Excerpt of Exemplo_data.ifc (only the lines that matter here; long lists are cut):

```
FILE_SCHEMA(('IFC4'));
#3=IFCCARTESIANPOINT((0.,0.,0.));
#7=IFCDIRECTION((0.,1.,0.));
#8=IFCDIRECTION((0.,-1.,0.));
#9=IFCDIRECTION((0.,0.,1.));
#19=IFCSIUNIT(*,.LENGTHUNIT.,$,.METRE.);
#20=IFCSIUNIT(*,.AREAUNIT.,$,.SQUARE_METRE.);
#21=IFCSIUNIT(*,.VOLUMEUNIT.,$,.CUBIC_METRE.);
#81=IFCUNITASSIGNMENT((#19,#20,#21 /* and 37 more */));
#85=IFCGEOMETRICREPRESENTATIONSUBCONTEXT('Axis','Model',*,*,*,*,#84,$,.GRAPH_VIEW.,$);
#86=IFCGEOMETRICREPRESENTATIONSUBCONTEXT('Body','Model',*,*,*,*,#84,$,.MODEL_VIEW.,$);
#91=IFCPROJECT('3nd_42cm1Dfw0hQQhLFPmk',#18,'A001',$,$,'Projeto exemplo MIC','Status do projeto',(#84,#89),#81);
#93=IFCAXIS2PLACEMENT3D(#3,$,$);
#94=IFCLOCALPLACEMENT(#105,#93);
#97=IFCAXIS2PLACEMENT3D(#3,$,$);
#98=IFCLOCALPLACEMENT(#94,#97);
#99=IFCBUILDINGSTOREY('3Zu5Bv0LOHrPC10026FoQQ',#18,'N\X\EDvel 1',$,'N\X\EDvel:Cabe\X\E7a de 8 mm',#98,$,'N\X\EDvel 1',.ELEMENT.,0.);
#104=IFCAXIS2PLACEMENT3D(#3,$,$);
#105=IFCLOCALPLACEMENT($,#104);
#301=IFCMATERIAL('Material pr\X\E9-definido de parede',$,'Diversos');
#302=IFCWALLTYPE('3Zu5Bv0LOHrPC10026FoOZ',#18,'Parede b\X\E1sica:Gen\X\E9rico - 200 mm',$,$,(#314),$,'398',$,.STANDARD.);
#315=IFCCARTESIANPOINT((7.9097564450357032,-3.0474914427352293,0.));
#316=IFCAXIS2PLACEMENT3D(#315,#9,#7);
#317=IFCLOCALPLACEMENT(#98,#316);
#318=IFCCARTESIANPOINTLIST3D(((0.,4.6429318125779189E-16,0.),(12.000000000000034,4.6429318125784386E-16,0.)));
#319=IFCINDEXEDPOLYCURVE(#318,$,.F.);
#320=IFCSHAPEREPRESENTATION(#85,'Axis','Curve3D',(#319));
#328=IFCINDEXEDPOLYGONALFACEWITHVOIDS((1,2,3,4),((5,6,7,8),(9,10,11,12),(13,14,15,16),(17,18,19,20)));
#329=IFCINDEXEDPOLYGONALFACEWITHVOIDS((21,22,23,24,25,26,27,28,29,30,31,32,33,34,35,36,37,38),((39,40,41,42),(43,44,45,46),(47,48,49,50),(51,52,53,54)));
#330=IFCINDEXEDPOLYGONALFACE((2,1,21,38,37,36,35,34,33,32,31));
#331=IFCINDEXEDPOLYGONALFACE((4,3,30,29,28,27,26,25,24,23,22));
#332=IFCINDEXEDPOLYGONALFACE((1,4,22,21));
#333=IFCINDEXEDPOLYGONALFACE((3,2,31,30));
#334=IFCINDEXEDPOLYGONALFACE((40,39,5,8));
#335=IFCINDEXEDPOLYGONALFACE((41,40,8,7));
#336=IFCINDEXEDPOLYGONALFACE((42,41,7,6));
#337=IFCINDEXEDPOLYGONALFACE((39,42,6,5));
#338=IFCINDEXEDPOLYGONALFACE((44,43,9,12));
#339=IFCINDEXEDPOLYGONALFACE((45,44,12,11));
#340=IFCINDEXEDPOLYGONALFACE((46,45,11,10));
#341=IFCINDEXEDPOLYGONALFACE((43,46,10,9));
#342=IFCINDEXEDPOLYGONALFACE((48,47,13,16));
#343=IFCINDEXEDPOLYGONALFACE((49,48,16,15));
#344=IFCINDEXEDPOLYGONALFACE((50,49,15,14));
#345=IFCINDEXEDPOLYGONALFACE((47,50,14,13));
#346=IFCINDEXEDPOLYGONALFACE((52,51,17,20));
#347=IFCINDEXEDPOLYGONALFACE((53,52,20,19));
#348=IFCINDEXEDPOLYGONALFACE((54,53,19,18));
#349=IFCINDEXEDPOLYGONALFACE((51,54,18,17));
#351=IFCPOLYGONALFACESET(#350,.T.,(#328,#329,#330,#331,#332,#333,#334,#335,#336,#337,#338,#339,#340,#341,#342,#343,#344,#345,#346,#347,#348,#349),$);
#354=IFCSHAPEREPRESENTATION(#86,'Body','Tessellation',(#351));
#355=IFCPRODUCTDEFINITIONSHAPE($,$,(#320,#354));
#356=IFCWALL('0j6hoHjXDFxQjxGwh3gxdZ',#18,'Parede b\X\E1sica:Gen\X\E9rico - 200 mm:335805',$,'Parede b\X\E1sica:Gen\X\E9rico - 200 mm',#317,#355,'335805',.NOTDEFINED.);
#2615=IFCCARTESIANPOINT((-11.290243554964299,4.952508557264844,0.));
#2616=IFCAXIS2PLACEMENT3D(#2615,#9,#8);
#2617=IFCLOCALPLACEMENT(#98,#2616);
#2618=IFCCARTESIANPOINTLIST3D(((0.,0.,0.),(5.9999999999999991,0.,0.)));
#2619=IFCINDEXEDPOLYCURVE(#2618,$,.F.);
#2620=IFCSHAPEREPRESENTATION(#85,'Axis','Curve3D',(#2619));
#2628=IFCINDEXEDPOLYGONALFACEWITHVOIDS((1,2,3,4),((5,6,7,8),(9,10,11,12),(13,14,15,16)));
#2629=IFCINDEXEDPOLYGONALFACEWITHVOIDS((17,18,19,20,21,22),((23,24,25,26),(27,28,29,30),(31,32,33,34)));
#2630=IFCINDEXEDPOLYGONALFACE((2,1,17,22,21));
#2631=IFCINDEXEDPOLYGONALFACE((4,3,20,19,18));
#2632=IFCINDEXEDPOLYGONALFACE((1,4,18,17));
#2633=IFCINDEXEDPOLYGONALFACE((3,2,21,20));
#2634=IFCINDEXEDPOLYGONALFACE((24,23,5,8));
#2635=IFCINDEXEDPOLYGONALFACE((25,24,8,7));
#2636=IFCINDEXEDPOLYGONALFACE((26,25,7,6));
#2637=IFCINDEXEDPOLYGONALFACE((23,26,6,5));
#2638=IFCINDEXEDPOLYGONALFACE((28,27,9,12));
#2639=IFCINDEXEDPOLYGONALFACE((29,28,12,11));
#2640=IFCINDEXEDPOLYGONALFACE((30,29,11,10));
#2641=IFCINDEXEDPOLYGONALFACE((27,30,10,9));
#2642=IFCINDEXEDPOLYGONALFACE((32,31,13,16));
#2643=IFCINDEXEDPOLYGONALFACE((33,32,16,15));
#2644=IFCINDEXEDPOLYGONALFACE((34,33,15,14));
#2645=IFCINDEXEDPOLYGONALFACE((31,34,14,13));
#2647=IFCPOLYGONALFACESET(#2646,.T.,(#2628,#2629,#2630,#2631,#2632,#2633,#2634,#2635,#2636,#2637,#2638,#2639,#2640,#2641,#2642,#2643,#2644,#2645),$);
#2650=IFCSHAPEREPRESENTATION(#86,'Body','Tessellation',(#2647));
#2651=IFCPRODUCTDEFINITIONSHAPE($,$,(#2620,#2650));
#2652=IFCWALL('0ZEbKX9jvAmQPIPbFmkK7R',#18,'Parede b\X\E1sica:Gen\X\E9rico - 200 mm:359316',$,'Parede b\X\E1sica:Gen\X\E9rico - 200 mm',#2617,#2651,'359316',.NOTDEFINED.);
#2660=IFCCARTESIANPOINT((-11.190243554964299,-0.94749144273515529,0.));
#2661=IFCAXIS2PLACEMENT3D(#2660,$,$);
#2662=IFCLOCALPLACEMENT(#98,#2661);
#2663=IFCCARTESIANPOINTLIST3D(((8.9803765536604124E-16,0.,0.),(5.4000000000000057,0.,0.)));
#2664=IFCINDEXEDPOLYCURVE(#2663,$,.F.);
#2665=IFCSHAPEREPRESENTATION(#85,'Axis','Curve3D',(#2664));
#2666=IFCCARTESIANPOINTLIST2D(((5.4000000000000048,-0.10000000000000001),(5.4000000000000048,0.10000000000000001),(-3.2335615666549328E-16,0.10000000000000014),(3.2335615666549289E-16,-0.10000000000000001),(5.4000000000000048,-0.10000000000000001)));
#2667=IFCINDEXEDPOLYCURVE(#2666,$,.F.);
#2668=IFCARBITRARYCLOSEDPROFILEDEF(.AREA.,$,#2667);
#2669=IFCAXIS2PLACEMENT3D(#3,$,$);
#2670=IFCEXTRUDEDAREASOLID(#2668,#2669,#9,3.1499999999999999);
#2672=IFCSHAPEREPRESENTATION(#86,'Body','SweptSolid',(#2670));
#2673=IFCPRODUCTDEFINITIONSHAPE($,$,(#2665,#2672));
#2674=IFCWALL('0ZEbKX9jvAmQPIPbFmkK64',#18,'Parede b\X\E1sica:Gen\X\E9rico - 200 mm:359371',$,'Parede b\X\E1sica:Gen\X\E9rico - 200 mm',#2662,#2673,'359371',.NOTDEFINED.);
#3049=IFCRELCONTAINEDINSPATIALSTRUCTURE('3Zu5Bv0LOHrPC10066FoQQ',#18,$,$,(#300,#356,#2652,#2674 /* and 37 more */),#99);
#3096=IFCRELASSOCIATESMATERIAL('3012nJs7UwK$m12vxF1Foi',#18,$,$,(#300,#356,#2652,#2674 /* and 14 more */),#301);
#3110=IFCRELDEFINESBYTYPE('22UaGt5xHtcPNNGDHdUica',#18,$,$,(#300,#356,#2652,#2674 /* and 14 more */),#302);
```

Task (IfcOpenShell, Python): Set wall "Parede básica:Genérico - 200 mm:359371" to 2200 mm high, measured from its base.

```python
import ifcopenshell
import ifcopenshell.geom
import ifcopenshell.util.representation
import ifcopenshell.util.shape

model = ifcopenshell.open("Exemplo_data.ifc")
settings = ifcopenshell.geom.settings()


def volume(element):
    """Net volume in cubic metres, openings subtracted."""
    shape = ifcopenshell.geom.create_shape(settings, element)
    return ifcopenshell.util.shape.get_volume(shape.geometry)


wall = model.by_guid("0ZEbKX9jvAmQPIPbFmkK64")
before = volume(wall)

body = ifcopenshell.util.representation.get_representation(wall, "Model", "Body")
solid = body.Items[0]
old_height = solid.Depth
solid.Depth = 2.2
after = volume(wall)

print(f"height {old_height:g} -> {solid.Depth:g}, volume {before:.3f} -> {after:.3f} m3")

model.write("Exemplo_data-out.ifc")
```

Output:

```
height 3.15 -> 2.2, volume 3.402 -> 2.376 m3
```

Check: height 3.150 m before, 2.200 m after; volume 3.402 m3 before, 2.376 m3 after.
